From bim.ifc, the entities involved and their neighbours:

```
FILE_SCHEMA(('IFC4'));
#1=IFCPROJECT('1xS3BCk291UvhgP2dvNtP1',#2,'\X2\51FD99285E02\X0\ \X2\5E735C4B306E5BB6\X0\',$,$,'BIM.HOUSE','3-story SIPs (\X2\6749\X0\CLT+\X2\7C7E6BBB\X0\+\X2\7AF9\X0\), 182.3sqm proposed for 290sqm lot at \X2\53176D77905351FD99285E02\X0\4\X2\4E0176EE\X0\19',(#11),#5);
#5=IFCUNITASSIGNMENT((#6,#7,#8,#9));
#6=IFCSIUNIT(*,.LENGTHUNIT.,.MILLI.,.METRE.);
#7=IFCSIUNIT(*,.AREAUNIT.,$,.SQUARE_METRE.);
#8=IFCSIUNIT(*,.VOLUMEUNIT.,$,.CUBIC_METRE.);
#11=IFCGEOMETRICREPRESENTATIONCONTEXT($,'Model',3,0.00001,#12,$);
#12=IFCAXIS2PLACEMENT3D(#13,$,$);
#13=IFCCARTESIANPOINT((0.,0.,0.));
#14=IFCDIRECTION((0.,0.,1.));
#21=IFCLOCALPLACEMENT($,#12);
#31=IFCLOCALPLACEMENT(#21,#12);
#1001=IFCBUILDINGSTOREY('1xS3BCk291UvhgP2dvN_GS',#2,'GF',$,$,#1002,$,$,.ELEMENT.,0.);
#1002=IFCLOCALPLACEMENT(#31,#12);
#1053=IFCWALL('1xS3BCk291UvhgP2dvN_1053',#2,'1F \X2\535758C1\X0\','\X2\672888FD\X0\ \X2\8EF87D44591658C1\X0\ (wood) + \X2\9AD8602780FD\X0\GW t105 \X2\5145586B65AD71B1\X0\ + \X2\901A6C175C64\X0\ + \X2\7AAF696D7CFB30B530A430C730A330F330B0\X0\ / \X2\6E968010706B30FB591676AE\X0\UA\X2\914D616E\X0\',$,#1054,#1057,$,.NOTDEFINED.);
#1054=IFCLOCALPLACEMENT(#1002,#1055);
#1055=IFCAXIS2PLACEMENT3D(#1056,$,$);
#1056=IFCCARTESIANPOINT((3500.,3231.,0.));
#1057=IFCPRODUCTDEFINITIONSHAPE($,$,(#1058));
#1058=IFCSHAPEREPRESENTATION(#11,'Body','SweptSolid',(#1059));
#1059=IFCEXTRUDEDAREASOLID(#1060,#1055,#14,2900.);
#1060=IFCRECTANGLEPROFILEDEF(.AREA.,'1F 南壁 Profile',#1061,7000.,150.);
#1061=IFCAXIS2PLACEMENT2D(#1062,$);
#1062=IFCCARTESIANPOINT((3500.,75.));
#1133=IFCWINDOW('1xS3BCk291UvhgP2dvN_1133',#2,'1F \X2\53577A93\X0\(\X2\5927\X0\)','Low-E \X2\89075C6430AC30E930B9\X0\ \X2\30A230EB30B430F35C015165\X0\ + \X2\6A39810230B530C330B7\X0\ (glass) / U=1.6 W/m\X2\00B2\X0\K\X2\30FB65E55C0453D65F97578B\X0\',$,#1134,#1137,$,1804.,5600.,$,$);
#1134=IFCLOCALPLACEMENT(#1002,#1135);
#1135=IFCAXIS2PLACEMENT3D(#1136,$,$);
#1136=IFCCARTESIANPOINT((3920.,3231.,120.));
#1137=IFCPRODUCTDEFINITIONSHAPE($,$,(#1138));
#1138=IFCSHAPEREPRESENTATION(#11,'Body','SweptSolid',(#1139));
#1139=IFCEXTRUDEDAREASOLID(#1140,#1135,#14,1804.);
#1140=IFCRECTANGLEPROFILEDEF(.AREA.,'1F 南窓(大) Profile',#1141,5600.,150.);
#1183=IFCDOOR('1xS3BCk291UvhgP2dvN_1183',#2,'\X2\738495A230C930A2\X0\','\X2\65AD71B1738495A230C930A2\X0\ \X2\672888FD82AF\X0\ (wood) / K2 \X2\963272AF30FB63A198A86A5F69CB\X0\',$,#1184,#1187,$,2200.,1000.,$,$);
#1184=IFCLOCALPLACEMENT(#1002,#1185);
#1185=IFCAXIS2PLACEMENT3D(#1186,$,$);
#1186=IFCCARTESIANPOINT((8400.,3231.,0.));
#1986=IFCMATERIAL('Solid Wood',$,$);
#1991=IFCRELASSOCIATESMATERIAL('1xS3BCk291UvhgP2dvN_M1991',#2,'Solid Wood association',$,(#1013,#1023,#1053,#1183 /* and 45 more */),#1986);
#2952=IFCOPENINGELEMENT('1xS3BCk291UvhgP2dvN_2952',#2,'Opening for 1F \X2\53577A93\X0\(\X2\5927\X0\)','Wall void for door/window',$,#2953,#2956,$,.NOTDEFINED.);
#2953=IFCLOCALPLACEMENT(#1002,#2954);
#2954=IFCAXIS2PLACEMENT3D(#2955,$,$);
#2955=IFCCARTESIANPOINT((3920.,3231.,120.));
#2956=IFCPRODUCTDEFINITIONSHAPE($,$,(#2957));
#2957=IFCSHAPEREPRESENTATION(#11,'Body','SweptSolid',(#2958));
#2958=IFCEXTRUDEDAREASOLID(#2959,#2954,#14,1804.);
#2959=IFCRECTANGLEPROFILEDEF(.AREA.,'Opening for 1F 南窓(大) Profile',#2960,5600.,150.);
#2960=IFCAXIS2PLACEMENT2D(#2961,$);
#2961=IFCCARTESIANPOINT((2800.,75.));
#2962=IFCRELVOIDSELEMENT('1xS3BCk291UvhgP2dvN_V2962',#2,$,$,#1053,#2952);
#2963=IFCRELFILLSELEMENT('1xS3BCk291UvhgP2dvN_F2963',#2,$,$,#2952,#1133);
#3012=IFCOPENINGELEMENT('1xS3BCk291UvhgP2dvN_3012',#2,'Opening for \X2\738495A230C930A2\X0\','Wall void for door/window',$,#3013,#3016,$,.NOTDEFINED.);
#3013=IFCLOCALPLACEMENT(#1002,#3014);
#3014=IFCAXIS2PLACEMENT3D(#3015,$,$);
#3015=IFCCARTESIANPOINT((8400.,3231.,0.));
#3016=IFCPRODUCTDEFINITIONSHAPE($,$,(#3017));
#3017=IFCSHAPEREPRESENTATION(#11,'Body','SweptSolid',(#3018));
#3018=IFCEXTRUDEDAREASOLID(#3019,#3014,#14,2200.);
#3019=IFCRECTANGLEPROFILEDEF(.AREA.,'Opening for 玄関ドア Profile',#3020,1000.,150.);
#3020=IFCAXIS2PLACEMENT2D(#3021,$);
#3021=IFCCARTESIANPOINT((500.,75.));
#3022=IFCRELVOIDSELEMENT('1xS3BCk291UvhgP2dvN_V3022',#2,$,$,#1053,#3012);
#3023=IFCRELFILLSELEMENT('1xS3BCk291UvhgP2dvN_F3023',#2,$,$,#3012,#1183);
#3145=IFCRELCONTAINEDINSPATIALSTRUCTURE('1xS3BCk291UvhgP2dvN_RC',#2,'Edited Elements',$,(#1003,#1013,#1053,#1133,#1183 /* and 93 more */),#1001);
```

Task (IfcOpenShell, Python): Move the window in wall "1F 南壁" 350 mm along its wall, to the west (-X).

```python
import ifcopenshell
import ifcopenshell.api.geometry
import ifcopenshell.util.placement

model = ifcopenshell.open("bim.ifc")

window = model.by_guid("1xS3BCk291UvhgP2dvN_1133")
opening = window.FillsVoids[0].RelatingOpeningElement
wall = opening.VoidsElements[0].RelatingBuildingElement

wall_matrix = ifcopenshell.util.placement.get_local_placement(wall.ObjectPlacement)
shift = wall_matrix[:3, 0] * -350.0
before = ifcopenshell.util.placement.get_local_placement(window.ObjectPlacement)[:3, 3].copy()

# The window is not placed relative to its opening, so move both.
for product in (opening, window):
    matrix = ifcopenshell.util.placement.get_local_placement(product.ObjectPlacement)
    matrix[:3, 3] += shift
    ifcopenshell.api.geometry.edit_object_placement(model, product=product, matrix=matrix, is_si=False)

after = ifcopenshell.util.placement.get_local_placement(window.ObjectPlacement)[:3, 3]
print("window moved by", (after - before).round(3) + 0.0)

model.write("bim-out.ifc")
```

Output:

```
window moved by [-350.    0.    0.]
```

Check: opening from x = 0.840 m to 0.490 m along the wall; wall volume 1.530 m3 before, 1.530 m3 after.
